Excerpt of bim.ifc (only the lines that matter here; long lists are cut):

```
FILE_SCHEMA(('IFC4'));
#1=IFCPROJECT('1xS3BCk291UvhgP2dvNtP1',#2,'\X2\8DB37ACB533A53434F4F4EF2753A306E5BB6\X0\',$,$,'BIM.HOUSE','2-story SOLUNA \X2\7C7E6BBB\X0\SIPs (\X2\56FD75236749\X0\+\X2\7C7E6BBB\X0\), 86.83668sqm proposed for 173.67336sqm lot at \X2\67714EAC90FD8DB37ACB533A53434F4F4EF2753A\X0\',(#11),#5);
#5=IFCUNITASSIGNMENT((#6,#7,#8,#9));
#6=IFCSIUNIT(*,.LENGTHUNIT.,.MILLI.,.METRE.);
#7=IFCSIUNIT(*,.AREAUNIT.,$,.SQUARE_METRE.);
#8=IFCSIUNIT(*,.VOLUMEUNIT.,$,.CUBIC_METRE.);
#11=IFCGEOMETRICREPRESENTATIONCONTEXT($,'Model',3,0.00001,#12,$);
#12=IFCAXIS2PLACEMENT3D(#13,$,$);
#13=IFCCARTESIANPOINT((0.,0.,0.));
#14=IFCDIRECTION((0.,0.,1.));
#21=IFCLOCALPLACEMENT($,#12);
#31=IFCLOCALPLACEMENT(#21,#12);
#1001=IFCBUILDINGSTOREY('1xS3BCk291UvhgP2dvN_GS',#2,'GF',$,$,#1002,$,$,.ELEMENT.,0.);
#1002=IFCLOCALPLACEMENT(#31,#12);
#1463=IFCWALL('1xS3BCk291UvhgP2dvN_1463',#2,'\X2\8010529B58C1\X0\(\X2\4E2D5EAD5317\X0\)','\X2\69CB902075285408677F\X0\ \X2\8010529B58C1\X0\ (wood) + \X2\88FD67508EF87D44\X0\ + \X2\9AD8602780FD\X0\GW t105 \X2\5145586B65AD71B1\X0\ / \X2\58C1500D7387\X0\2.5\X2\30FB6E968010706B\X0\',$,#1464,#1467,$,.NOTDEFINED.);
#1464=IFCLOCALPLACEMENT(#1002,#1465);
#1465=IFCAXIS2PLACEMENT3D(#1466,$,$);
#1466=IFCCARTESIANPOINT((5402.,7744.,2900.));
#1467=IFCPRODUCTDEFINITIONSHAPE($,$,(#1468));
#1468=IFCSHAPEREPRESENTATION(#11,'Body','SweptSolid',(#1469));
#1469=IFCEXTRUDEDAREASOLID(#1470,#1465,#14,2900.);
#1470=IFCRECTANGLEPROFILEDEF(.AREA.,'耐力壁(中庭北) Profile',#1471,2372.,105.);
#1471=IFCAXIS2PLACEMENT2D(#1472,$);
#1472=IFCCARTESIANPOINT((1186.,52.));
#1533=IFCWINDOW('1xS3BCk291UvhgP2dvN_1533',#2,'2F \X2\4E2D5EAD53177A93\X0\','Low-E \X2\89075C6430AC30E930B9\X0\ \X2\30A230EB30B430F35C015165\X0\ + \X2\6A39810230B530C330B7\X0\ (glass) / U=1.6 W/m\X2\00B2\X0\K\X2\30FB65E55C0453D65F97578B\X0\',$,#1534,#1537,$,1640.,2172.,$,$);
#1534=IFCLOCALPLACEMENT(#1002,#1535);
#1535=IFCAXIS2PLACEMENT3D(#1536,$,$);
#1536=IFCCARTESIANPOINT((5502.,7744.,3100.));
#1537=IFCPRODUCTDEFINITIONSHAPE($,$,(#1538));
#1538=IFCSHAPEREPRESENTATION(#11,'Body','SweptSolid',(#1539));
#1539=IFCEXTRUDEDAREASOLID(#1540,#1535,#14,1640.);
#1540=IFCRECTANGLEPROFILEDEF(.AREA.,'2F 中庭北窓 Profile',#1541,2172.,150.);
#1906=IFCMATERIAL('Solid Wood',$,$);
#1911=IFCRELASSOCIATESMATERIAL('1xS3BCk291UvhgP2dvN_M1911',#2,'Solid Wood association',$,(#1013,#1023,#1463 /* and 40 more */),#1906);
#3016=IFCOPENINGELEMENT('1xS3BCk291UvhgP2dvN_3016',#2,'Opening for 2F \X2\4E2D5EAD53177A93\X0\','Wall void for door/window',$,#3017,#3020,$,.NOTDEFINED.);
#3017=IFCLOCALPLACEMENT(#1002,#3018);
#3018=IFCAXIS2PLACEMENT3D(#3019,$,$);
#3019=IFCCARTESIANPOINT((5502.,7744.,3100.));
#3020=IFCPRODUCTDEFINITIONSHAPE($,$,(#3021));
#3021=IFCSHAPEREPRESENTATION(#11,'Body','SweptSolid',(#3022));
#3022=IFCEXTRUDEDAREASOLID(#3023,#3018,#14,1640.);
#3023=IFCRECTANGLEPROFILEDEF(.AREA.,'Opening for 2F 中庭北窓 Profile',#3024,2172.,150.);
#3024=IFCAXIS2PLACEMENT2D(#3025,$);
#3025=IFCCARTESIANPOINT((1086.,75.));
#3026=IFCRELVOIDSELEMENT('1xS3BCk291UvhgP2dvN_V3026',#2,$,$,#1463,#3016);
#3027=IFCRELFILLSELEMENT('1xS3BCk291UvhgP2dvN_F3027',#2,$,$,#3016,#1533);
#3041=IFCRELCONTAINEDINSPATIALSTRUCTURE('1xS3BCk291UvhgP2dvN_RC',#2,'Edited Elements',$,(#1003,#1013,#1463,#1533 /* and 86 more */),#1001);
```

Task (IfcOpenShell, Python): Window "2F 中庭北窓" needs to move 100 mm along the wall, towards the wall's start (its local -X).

```python
import ifcopenshell
import ifcopenshell.api.geometry
import ifcopenshell.util.placement
import ifcopenshell.util.unit

model = ifcopenshell.open("bim.ifc")
unit_scale = ifcopenshell.util.unit.calculate_unit_scale(model)

window = model.by_guid("1xS3BCk291UvhgP2dvN_1533")
opening = window.FillsVoids[0].RelatingOpeningElement
wall = opening.VoidsElements[0].RelatingBuildingElement

wall_matrix = ifcopenshell.util.placement.get_local_placement(wall.ObjectPlacement)
shift = wall_matrix[:3, 0] * -0.1 / unit_scale
before = ifcopenshell.util.placement.get_local_placement(window.ObjectPlacement)[:3, 3].copy()

# The window is not placed relative to its opening, so move both.
for product in (opening, window):
    matrix = ifcopenshell.util.placement.get_local_placement(product.ObjectPlacement)
    matrix[:3, 3] += shift
    ifcopenshell.api.geometry.edit_object_placement(model, product=product, matrix=matrix, is_si=False)

after = ifcopenshell.util.placement.get_local_placement(window.ObjectPlacement)[:3, 3]
print("window moved by", (after - before).round(3) + 0.0)

model.write("bim_updated.ifc")
```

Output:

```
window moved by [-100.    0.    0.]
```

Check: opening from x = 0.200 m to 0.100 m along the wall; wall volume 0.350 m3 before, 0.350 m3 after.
